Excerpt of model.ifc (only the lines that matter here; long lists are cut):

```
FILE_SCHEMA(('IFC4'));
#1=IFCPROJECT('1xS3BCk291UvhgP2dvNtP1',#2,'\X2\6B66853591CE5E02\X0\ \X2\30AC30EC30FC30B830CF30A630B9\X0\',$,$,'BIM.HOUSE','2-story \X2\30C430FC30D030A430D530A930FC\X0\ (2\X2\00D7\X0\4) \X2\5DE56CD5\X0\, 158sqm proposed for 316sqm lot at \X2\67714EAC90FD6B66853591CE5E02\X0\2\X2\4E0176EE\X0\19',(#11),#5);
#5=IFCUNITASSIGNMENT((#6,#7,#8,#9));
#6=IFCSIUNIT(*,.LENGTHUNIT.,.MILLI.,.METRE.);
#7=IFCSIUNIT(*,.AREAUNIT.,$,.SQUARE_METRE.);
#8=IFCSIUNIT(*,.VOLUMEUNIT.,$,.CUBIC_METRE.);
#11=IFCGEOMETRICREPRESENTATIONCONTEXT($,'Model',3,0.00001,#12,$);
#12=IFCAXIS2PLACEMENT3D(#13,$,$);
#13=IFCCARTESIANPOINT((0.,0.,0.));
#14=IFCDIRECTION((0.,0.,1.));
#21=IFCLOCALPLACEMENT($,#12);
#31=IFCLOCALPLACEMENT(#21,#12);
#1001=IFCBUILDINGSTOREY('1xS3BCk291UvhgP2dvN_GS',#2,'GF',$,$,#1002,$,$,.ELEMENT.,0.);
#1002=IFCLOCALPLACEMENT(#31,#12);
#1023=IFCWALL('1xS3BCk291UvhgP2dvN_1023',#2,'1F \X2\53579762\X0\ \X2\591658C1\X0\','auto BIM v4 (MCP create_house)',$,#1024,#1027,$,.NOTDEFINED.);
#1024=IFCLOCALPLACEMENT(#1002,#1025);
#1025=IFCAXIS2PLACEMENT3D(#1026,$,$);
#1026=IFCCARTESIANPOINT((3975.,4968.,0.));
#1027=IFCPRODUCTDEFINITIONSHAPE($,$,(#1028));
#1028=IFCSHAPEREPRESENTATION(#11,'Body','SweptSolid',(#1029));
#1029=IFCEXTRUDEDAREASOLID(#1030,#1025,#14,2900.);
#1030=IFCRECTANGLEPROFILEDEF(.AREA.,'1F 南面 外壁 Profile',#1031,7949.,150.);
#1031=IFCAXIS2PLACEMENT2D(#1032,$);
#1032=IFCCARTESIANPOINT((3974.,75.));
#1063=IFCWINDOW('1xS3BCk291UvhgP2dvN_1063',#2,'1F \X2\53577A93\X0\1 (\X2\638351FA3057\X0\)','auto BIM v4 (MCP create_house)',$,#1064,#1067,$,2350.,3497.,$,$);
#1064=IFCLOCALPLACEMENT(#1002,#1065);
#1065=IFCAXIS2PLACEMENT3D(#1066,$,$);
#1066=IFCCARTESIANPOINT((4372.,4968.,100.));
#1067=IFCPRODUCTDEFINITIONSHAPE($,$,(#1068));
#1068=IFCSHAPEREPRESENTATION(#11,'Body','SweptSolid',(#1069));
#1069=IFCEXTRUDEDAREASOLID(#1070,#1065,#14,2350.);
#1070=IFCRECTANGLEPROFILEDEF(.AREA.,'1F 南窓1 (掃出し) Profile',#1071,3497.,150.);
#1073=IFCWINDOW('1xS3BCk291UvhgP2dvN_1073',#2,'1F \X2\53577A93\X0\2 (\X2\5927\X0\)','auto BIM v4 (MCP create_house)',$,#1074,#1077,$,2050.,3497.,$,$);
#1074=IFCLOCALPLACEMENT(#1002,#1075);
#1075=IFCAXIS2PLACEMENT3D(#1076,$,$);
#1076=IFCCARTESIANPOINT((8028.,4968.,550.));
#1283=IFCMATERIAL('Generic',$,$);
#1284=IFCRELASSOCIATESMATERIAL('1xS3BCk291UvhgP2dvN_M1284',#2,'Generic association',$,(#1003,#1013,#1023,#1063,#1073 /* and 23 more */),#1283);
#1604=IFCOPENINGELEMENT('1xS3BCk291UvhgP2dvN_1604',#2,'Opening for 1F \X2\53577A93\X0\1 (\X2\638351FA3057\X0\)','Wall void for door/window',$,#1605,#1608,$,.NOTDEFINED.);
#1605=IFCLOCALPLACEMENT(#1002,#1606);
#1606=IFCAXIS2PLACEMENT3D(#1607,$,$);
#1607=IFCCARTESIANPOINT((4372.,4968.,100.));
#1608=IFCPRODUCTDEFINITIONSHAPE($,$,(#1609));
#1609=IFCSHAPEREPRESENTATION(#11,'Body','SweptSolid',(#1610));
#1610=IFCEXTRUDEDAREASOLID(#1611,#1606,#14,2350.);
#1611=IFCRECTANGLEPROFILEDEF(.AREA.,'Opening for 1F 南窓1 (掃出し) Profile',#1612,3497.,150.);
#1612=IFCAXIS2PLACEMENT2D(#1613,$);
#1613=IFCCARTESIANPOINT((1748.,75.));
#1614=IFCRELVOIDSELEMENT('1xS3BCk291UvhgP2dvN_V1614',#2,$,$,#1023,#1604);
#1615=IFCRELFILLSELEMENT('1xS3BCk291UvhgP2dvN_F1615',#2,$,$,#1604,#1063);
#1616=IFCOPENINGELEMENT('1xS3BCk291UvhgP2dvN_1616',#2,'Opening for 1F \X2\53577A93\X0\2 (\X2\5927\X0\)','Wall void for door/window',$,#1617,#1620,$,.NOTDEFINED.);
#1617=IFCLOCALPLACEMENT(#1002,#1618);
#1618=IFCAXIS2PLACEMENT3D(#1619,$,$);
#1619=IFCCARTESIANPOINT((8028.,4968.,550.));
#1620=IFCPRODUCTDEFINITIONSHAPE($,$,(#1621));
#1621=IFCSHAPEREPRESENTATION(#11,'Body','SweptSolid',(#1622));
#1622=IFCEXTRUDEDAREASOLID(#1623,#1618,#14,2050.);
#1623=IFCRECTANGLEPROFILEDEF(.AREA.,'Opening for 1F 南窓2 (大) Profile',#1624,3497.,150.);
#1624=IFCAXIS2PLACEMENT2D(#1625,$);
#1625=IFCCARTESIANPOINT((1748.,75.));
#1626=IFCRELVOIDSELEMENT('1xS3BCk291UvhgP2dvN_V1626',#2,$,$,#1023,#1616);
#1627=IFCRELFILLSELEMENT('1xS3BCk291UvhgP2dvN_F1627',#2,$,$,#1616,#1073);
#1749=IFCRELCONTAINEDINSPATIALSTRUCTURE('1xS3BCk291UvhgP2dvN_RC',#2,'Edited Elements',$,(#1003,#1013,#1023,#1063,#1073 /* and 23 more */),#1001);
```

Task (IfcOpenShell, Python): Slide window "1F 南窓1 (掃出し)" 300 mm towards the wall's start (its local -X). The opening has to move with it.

```python
import ifcopenshell
import ifcopenshell.api.geometry
import ifcopenshell.util.placement

model = ifcopenshell.open("model.ifc")

window = model.by_id(1063)
opening = window.FillsVoids[0].RelatingOpeningElement
wall = opening.VoidsElements[0].RelatingBuildingElement

wall_matrix = ifcopenshell.util.placement.get_local_placement(wall.ObjectPlacement)
shift = wall_matrix[:3, 0] * -300.0
before = ifcopenshell.util.placement.get_local_placement(window.ObjectPlacement)[:3, 3].copy()

# The window is not placed relative to its opening, so move both.
for product in (opening, window):
    matrix = ifcopenshell.util.placement.get_local_placement(product.ObjectPlacement)
    matrix[:3, 3] += shift
    ifcopenshell.api.geometry.edit_object_placement(model, product=product, matrix=matrix, is_si=False)

after = ifcopenshell.util.placement.get_local_placement(window.ObjectPlacement)[:3, 3]
print("window moved by", (after - before).round(3) + 0.0)

model.write("model_updated.ifc")
```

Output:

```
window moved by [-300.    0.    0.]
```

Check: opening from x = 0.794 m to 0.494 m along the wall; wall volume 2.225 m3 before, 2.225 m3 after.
